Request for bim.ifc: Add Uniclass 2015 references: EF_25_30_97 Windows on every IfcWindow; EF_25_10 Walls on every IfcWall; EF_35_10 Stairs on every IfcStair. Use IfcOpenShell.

First a look at what the model holds.

```python
import ifcopenshell

model = ifcopenshell.open("bim.ifc")
print(model.schema)
print("classifications:", [c.Name for c in model.by_type("IfcClassification")])
for ifc_class in ("IfcDoor", "IfcRoof", "IfcStair", "IfcWall", "IfcWindow"):
    print(ifc_class, len(model.by_type(ifc_class)))
```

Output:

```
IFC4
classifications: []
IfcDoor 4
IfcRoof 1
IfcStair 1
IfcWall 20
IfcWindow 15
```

```python
import ifcopenshell
import ifcopenshell.api.classification

model = ifcopenshell.open("bim.ifc")

system = ifcopenshell.api.classification.add_classification(model, classification="Uniclass 2015")

codes = {
    "IfcWindow": ("EF_25_30_97", "Windows"),
    "IfcWall": ("EF_25_10", "Walls"),
    "IfcStair": ("EF_35_10", "Stairs"),
}
for ifc_class, (code, name) in codes.items():
    products = model.by_type(ifc_class)
    ifcopenshell.api.classification.add_reference(
        model, products=products, classification=system, identification=code, name=name
    )
    print(code, len(products))

model.write("bim-out.ifc")
```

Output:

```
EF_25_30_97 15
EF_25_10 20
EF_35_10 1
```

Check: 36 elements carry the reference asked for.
